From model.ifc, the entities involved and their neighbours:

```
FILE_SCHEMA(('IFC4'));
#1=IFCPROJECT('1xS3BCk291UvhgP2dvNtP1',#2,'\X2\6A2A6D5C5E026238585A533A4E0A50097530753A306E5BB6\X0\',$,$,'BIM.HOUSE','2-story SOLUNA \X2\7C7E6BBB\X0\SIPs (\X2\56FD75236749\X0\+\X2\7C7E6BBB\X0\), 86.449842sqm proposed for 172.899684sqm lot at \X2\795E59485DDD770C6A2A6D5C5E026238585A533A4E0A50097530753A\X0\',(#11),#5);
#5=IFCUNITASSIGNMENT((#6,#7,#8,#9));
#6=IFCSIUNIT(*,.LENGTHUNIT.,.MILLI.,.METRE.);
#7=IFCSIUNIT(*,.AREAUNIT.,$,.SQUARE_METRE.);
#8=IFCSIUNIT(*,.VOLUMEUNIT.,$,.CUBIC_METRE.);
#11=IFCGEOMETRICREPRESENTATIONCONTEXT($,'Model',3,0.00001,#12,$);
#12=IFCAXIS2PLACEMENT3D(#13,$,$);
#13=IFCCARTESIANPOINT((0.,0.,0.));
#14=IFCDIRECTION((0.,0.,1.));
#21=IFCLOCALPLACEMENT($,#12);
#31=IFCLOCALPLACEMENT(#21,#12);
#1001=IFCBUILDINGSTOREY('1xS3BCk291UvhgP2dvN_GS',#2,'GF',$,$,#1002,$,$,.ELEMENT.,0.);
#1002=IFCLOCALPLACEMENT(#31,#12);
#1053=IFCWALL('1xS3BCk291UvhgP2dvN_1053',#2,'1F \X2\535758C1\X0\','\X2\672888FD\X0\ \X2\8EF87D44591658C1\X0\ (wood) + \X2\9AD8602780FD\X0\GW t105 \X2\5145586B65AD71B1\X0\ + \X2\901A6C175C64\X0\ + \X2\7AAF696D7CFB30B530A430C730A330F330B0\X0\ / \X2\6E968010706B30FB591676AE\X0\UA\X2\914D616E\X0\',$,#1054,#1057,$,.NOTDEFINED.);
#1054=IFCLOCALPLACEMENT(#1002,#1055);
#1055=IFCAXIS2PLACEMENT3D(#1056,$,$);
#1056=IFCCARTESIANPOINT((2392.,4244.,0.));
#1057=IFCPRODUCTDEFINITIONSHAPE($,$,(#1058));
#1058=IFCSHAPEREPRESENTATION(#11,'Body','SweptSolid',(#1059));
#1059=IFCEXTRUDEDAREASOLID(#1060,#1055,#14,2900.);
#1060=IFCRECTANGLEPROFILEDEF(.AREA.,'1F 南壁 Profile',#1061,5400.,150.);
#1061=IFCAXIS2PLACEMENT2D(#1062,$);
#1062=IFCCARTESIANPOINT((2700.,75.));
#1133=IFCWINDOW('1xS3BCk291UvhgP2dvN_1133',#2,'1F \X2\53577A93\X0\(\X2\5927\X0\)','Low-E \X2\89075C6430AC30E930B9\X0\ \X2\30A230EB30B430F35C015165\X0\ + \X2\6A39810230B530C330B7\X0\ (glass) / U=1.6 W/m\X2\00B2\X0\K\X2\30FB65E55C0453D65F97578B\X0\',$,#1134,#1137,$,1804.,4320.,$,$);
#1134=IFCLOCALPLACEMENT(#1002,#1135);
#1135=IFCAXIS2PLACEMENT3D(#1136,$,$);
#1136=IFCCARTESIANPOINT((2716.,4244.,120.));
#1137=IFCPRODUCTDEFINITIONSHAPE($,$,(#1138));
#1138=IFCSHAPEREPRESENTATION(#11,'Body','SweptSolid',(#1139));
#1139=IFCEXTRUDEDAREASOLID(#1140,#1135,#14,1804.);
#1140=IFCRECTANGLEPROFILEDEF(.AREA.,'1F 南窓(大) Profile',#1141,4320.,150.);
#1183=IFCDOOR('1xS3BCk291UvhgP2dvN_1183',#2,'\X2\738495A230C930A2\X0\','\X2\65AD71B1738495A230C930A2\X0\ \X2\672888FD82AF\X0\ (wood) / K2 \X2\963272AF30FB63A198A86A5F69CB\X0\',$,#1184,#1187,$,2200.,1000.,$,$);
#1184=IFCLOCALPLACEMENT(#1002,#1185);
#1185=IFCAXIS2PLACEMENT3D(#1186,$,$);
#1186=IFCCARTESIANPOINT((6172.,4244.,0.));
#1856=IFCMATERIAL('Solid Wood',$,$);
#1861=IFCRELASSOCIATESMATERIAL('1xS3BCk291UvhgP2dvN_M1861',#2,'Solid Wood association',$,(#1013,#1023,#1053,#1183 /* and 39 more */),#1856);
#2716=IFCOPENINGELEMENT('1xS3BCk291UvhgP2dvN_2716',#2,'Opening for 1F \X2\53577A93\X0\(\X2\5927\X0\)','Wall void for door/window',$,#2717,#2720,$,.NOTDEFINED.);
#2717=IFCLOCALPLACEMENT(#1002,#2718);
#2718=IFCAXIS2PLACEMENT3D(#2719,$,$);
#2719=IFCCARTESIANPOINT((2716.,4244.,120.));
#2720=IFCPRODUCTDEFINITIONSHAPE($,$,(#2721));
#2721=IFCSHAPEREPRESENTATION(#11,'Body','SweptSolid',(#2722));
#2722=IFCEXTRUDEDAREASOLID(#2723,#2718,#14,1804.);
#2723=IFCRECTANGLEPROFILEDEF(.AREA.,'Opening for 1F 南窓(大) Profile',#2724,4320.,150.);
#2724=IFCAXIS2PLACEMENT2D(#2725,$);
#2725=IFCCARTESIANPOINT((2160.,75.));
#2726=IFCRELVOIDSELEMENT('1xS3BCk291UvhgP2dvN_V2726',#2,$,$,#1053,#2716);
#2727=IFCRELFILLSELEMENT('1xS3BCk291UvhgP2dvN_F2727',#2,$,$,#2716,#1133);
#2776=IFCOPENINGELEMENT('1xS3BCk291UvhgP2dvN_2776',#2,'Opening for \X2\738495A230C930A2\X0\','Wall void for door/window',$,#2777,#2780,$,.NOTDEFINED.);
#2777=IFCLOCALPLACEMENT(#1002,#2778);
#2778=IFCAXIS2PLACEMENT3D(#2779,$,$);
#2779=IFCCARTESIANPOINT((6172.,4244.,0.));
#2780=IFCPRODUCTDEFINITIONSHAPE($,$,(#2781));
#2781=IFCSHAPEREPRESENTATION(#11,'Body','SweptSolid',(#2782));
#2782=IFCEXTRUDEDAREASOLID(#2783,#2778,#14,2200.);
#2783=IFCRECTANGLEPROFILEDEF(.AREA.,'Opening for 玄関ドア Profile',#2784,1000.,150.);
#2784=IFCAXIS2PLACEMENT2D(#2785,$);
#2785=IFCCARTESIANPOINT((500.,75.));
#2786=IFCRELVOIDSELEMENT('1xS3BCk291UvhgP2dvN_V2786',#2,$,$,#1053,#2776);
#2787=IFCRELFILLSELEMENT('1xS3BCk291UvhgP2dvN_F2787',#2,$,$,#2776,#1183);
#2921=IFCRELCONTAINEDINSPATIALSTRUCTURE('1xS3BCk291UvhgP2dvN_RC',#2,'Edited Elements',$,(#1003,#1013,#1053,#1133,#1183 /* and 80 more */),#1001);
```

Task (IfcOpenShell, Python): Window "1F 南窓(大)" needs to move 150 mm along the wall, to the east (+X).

```python
import ifcopenshell
import ifcopenshell.api.geometry
import ifcopenshell.util.placement

model = ifcopenshell.open("model.ifc")

window = model.by_guid("1xS3BCk291UvhgP2dvN_1133")
opening = window.FillsVoids[0].RelatingOpeningElement
wall = opening.VoidsElements[0].RelatingBuildingElement

wall_matrix = ifcopenshell.util.placement.get_local_placement(wall.ObjectPlacement)
shift = wall_matrix[:3, 0] * 150.0
before = ifcopenshell.util.placement.get_local_placement(window.ObjectPlacement)[:3, 3].copy()

# The window is not placed relative to its opening, so move both.
for product in (opening, window):
    matrix = ifcopenshell.util.placement.get_local_placement(product.ObjectPlacement)
    matrix[:3, 3] += shift
    ifcopenshell.api.geometry.edit_object_placement(model, product=product, matrix=matrix, is_si=False)

after = ifcopenshell.util.placement.get_local_placement(window.ObjectPlacement)[:3, 3]
print("window moved by", (after - before).round(3) + 0.0)

model.write("model-out.ifc")
```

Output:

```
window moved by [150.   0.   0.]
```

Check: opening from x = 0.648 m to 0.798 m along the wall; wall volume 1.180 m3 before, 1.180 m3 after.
